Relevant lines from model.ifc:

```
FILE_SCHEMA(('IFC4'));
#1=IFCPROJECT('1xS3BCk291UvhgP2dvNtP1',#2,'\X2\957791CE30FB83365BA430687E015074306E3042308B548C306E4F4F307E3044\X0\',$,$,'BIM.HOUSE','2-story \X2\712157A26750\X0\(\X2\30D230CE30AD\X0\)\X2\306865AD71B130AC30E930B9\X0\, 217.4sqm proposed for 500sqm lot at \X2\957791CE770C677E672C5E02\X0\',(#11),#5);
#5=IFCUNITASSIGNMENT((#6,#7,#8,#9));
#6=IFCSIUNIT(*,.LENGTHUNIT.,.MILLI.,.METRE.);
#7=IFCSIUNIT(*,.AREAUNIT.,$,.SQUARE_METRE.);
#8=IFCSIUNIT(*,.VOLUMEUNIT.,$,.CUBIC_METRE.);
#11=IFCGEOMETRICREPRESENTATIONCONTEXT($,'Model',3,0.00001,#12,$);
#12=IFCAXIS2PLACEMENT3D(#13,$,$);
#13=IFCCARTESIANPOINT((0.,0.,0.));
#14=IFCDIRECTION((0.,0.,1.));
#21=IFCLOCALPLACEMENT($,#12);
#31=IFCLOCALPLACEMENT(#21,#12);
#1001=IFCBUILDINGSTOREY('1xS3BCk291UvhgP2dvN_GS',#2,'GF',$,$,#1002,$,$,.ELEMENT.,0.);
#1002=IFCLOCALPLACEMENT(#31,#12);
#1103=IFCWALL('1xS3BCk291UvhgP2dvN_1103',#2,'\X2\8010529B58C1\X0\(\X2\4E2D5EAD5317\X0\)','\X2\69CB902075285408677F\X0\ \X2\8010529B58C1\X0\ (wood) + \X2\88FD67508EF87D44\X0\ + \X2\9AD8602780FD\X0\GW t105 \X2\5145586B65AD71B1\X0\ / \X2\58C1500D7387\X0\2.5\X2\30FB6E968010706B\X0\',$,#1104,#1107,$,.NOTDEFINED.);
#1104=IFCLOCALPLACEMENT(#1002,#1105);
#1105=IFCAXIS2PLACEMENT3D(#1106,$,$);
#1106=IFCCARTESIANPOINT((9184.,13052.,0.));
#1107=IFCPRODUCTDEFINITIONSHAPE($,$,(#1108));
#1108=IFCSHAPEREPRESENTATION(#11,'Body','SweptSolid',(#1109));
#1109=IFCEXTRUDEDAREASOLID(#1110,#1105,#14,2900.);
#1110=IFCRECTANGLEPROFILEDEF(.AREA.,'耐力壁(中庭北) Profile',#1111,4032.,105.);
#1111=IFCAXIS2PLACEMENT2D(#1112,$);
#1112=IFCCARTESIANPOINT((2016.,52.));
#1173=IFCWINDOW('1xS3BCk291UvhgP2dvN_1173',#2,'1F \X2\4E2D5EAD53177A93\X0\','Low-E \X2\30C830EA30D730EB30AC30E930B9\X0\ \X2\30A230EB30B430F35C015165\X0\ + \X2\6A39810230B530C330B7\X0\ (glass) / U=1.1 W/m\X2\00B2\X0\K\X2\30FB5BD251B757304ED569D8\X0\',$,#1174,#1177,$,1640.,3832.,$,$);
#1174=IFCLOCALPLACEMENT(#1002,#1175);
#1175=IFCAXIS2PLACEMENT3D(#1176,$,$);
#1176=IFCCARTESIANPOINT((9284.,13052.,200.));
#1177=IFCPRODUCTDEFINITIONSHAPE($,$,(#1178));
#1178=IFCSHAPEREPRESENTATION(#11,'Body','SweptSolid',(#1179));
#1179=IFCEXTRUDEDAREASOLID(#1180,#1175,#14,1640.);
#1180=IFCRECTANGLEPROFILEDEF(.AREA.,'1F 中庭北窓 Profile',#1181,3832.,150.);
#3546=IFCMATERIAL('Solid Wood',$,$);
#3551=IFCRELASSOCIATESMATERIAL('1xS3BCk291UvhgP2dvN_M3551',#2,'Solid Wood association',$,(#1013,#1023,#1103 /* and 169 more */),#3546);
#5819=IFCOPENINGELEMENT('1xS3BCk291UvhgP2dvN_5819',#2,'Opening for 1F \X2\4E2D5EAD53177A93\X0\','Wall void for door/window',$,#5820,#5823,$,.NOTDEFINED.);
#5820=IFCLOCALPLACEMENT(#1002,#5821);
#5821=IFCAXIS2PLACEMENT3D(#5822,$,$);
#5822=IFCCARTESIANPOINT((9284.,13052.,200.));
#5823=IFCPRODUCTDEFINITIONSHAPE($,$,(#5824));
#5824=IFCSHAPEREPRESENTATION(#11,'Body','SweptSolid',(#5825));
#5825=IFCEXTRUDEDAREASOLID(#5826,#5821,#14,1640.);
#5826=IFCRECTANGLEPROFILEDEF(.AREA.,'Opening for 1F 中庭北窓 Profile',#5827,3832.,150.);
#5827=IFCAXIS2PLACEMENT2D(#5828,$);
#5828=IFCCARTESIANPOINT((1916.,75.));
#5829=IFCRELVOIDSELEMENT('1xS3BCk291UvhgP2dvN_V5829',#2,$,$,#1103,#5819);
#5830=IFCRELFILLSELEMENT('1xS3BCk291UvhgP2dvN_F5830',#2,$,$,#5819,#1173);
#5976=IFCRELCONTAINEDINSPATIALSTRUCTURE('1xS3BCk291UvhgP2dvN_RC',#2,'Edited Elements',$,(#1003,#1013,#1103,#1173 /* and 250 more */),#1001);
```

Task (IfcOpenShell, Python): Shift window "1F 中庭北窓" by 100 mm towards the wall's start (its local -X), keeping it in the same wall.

```python
import ifcopenshell
import ifcopenshell.api.geometry
import ifcopenshell.util.placement
import ifcopenshell.util.unit

model = ifcopenshell.open("model.ifc")
unit_scale = ifcopenshell.util.unit.calculate_unit_scale(model)

window = model.by_guid("1xS3BCk291UvhgP2dvN_1173")
opening = window.FillsVoids[0].RelatingOpeningElement
wall = opening.VoidsElements[0].RelatingBuildingElement

wall_matrix = ifcopenshell.util.placement.get_local_placement(wall.ObjectPlacement)
shift = wall_matrix[:3, 0] * -0.1 / unit_scale
before = ifcopenshell.util.placement.get_local_placement(window.ObjectPlacement)[:3, 3].copy()

# The window is not placed relative to its opening, so move both.
for product in (opening, window):
    matrix = ifcopenshell.util.placement.get_local_placement(product.ObjectPlacement)
    matrix[:3, 3] += shift
    ifcopenshell.api.geometry.edit_object_placement(model, product=product, matrix=matrix, is_si=False)

after = ifcopenshell.util.placement.get_local_placement(window.ObjectPlacement)[:3, 3]
print("window moved by", (after - before).round(3) + 0.0)

model.write("model_edited.ifc")
```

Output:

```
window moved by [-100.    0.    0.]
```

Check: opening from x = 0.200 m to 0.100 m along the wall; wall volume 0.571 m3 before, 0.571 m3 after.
